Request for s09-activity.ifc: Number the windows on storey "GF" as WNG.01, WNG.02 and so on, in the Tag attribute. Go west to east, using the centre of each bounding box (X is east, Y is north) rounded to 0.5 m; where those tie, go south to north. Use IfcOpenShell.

First a look at what the model holds.

```python
import ifcopenshell
import ifcopenshell.util.element
import ifcopenshell.util.placement

model = ifcopenshell.open("s09-activity.ifc")
print(model.schema)
storey = next(s for s in model.by_type("IfcBuildingStorey") if s.Name == "GF")
windows = [e for e in ifcopenshell.util.element.get_decomposition(storey) if e.is_a("IfcWindow")]
for e in sorted(windows, key=lambda e: e.id()):
    origin = ifcopenshell.util.placement.get_local_placement(e.ObjectPlacement)[:3, 3]
    print(e.id(), e.Tag, e.Name, origin.round(2) + 0.0, sep=" | ")
```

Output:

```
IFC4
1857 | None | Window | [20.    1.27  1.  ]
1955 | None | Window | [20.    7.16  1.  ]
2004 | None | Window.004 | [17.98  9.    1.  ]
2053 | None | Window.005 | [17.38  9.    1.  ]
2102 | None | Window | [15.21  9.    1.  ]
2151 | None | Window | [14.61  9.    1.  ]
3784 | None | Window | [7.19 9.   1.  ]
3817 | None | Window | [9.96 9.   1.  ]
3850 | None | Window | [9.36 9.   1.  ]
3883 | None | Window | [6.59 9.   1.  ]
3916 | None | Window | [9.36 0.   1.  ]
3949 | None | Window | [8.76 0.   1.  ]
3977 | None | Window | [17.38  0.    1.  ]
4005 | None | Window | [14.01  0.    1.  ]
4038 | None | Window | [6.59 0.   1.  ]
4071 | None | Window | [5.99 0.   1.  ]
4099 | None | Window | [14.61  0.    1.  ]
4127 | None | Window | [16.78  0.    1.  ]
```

```python
import ifcopenshell
import ifcopenshell.geom
import ifcopenshell.util.element
import ifcopenshell.util.shape

model = ifcopenshell.open("s09-activity.ifc")
settings = ifcopenshell.geom.settings()
settings.set("use-world-coords", True)


def centre(element):
    shape = ifcopenshell.geom.create_shape(settings, element)
    return ifcopenshell.util.shape.get_bbox_centroid(shape.geometry)


storey = next(s for s in model.by_type("IfcBuildingStorey") if s.Name == "GF")
windows = [e for e in ifcopenshell.util.element.get_decomposition(storey) if e.is_a("IfcWindow")]

# Insertion points can sit at a corner or the storey origin, so sort by the geometry (in metres).
centres = {e: centre(e) for e in windows}
windows.sort(key=lambda e: (round(centres[e][0] / 0.5), centres[e][1]))

for i, e in enumerate(windows, start=1):
    number = f"WNG.{i:02d}"
    e.Tag = number
    print(e.id(), number)

model.write("s09-activity-out.ifc")
```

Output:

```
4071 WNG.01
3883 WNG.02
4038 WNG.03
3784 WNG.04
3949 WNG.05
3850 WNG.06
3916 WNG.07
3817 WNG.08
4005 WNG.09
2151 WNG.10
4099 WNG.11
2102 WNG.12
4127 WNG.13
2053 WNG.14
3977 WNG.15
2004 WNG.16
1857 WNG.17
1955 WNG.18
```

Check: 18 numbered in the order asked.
